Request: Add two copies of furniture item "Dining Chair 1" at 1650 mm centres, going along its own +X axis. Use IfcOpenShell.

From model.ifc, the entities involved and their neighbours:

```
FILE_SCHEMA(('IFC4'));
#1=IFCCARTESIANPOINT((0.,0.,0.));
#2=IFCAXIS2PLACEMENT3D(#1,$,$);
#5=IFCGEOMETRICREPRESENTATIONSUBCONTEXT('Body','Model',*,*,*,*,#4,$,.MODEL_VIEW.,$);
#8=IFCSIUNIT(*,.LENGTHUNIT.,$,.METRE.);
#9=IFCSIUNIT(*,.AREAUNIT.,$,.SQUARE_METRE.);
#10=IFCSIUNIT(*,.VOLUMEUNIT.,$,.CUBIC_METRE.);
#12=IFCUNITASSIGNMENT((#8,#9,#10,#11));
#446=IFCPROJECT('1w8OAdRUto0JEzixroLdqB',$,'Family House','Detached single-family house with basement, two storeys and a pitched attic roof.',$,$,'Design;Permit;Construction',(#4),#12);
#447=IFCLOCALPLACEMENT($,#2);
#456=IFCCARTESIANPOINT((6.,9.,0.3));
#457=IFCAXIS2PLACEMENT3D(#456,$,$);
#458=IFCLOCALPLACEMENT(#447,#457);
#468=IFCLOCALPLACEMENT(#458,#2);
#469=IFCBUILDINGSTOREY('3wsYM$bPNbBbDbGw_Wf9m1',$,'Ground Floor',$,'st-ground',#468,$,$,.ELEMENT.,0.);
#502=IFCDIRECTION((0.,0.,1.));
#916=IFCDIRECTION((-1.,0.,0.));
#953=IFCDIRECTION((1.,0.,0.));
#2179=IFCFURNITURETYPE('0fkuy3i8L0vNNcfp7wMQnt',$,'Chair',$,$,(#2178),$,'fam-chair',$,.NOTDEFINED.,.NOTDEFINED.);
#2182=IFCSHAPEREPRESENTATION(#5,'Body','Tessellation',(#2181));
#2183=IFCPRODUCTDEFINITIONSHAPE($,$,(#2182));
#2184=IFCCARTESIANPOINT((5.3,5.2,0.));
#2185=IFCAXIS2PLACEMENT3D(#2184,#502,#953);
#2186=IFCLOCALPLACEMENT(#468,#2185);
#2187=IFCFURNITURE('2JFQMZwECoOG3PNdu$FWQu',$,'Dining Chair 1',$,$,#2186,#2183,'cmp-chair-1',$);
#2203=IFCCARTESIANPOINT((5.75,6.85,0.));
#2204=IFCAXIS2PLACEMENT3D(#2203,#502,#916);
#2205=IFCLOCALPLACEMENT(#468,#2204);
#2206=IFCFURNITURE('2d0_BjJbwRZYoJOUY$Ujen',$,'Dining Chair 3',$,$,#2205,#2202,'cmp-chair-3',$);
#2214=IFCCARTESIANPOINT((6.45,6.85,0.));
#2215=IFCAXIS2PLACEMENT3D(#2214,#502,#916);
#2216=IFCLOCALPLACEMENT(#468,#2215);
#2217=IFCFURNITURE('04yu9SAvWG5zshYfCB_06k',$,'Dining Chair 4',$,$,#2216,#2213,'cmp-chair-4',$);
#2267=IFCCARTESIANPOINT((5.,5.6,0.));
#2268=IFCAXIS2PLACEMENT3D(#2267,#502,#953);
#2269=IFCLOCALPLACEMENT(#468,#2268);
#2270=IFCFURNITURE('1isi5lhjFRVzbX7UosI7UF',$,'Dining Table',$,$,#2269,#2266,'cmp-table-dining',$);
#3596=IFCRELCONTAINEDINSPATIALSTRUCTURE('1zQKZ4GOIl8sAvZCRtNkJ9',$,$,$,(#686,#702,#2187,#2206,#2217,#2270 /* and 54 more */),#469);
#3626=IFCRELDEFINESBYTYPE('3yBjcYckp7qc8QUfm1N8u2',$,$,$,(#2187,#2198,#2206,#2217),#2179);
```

```python
import ifcopenshell
import ifcopenshell.api.geometry
import ifcopenshell.api.root
import ifcopenshell.util.element
import ifcopenshell.util.placement
import ifcopenshell.util.unit

model = ifcopenshell.open("model.ifc")
unit_scale = ifcopenshell.util.unit.calculate_unit_scale(model)

source = model.by_id(2187)
base = ifcopenshell.util.placement.get_local_placement(source.ObjectPlacement)
step = base[:3, 0] * 1.65 / unit_scale

for i in range(1, 3):
    copy = ifcopenshell.api.root.copy_class(model, product=source)
    copy.Representation = ifcopenshell.util.element.copy_deep(
        model, source.Representation, exclude=["IfcGeometricRepresentationContext", "IfcRepresentationMap"]
    )
    copy.Tag = None
    matrix = base.copy()
    matrix[:3, 3] += i * step
    print("added at", matrix[:3, 3].round(3) + 0.0)
    ifcopenshell.api.geometry.edit_object_placement(model, product=copy, matrix=matrix, is_si=False)

model.write("model_rev.ifc")
```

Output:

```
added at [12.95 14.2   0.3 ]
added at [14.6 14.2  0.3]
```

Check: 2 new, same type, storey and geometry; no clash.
